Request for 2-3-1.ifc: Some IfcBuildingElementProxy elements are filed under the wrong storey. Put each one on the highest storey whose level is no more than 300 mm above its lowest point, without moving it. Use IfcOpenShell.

First a look at what the model holds.

```python
import ifcopenshell
import ifcopenshell.util.element
import ifcopenshell.util.placement

model = ifcopenshell.open("2-3-1.ifc")
print(model.schema)
for storey in model.by_type("IfcBuildingStorey"):
    level = ifcopenshell.util.placement.get_storey_elevation(storey)
    count = sum(e.is_a("IfcBuildingElementProxy") for e in ifcopenshell.util.element.get_contained(storey))
    print(storey.id(), storey.Name, round(level, 3), count, sep=" | ")
```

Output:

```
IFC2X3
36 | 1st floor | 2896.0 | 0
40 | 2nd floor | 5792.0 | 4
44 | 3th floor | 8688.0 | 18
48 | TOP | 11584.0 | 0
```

```python
import ifcopenshell
import ifcopenshell.api.spatial
import ifcopenshell.geom
import ifcopenshell.util.element
import ifcopenshell.util.placement
import ifcopenshell.util.shape
import ifcopenshell.util.unit

model = ifcopenshell.open("2-3-1.ifc")
unit_scale = ifcopenshell.util.unit.calculate_unit_scale(model)
settings = ifcopenshell.geom.settings()

levels = sorted(
    ((ifcopenshell.util.placement.get_storey_elevation(s) * unit_scale, s) for s in model.by_type("IfcBuildingStorey")),
    key=lambda pair: pair[0],
)

for e in model.by_type("IfcBuildingElementProxy"):
    current = e.ContainedInStructure[0].RelatingStructure if e.ContainedInStructure else None
    if current is None or not current.is_a("IfcBuildingStorey"):
        continue
    shape = ifcopenshell.geom.create_shape(settings, e)
    bottom = ifcopenshell.util.shape.get_shape_bottom_elevation(shape, shape.geometry)
    below = [s for level, s in levels if level <= bottom + 0.3]
    storey = below[-1] if below else levels[0][1]
    if storey != current:
        # assign_container keeps the world position.
        ifcopenshell.api.spatial.assign_container(model, products=[e], relating_structure=storey)
        print(e.id(), current.Name, "->", storey.Name)

model.write("2-3-1_edited.ifc")
```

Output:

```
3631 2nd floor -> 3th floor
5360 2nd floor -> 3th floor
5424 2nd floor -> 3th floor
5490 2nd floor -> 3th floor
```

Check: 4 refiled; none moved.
